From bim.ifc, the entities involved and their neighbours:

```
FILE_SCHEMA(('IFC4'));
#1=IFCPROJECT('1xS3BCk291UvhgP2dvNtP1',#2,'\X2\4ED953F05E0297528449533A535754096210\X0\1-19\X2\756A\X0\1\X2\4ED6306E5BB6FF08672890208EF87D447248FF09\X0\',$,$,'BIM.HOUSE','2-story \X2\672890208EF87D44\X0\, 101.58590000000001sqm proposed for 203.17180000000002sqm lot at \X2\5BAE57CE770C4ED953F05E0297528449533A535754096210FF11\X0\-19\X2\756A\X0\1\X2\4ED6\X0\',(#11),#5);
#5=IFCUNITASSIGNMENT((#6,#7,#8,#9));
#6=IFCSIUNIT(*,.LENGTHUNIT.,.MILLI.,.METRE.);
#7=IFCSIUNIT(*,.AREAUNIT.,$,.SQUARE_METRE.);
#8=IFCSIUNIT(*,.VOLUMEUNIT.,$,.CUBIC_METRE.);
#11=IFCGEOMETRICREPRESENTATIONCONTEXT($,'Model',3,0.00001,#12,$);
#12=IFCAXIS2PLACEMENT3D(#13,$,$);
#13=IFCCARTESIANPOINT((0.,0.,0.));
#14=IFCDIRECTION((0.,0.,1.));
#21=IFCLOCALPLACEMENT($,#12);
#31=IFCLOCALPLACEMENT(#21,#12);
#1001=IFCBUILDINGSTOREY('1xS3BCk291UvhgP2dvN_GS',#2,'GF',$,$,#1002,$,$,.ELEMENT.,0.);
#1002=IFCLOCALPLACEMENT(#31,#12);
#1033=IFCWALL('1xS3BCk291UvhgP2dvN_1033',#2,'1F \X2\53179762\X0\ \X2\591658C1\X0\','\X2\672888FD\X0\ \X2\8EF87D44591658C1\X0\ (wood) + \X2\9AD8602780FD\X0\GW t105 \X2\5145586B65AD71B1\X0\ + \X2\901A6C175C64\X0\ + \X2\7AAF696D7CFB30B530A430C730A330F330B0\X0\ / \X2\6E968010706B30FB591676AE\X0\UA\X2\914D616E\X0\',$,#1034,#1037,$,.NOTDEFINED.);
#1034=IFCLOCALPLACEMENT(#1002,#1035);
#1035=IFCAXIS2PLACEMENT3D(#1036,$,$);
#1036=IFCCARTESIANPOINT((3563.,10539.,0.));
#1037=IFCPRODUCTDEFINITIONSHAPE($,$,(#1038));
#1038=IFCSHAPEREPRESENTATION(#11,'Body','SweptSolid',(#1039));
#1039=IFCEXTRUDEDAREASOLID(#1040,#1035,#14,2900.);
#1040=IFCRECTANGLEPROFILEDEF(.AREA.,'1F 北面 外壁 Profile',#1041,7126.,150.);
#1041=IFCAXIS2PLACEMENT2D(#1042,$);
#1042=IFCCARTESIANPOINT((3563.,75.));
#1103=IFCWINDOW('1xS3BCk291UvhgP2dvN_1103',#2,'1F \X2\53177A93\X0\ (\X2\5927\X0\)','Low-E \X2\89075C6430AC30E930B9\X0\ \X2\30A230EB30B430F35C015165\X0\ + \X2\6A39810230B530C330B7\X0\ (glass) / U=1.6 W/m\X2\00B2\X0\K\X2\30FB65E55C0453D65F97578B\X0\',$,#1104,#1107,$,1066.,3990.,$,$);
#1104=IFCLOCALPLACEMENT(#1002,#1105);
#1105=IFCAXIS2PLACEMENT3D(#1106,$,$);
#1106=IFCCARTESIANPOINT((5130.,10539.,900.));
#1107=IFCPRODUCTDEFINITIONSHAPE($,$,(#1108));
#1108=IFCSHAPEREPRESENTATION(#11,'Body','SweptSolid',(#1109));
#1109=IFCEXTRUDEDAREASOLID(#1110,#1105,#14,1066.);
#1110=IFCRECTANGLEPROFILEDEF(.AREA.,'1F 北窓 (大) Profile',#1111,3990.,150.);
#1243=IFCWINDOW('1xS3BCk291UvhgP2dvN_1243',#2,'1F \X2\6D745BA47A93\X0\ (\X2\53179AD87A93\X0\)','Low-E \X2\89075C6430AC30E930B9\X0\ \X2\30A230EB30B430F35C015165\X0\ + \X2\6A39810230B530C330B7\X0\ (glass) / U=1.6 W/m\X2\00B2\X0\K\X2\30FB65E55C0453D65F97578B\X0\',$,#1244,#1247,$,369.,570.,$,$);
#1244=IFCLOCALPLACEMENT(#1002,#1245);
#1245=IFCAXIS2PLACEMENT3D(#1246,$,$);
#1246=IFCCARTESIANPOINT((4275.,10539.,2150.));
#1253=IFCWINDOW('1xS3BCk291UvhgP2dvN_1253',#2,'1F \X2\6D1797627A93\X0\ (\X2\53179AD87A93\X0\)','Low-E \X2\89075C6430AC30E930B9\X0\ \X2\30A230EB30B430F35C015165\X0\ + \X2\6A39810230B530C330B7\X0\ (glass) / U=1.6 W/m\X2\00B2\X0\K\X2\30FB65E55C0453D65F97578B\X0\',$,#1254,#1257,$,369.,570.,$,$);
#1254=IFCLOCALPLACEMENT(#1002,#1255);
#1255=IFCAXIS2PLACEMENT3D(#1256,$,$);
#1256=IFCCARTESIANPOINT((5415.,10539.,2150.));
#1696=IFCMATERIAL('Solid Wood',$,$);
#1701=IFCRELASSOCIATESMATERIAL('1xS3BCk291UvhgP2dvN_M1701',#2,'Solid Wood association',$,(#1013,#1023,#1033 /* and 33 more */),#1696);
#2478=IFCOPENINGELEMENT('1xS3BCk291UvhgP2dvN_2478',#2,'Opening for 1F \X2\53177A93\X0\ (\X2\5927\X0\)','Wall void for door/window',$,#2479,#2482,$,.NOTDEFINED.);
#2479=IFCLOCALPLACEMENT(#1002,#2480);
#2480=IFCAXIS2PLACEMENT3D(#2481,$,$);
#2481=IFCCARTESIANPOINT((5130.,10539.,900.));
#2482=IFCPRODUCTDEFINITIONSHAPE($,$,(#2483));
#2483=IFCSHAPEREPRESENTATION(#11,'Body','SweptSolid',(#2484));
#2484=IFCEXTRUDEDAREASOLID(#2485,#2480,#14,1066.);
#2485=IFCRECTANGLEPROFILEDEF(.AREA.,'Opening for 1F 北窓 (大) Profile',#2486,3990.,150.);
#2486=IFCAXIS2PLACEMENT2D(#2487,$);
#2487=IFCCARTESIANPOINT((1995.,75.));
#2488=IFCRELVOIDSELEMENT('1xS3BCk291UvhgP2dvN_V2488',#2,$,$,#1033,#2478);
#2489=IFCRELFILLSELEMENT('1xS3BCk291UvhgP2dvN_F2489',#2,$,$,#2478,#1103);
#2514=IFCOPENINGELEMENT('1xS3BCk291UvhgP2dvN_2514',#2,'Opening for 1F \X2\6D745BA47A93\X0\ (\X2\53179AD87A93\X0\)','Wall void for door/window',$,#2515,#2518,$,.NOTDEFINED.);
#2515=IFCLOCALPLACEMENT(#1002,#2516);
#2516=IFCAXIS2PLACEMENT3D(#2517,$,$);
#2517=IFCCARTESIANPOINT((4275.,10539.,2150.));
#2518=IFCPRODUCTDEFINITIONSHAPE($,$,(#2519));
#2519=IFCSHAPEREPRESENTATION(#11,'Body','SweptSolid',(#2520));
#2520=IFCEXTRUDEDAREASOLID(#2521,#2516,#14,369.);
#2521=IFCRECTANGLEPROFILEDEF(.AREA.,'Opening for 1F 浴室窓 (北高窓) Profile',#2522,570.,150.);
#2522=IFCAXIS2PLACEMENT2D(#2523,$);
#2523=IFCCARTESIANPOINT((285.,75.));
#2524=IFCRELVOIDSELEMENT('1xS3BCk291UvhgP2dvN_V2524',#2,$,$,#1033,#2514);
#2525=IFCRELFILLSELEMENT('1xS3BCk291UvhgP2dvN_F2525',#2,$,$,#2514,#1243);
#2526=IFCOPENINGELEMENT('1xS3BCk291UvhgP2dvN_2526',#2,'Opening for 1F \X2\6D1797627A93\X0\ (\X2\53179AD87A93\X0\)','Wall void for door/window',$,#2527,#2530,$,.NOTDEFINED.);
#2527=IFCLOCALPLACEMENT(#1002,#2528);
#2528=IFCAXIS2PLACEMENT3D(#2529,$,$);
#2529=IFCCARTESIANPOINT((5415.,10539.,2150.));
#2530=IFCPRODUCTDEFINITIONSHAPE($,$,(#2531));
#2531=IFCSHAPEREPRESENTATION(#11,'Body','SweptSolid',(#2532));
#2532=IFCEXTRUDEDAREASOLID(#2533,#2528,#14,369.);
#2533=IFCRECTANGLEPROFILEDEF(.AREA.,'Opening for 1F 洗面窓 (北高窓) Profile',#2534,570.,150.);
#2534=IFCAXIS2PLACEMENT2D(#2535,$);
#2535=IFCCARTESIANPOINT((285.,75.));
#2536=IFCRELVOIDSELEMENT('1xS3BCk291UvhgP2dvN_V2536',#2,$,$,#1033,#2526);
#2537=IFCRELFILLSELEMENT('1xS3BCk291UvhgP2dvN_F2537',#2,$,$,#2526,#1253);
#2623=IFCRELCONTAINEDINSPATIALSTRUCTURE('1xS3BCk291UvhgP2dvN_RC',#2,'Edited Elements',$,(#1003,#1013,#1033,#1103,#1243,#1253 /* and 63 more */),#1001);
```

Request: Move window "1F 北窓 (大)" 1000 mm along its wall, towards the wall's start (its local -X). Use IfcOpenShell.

```python
import ifcopenshell
import ifcopenshell.api.geometry
import ifcopenshell.util.placement
import ifcopenshell.util.unit

model = ifcopenshell.open("bim.ifc")
unit_scale = ifcopenshell.util.unit.calculate_unit_scale(model)

window = model.by_guid("1xS3BCk291UvhgP2dvN_1103")
opening = window.FillsVoids[0].RelatingOpeningElement
wall = opening.VoidsElements[0].RelatingBuildingElement

wall_matrix = ifcopenshell.util.placement.get_local_placement(wall.ObjectPlacement)
shift = wall_matrix[:3, 0] * -1 / unit_scale
before = ifcopenshell.util.placement.get_local_placement(window.ObjectPlacement)[:3, 3].copy()

# The window is not placed relative to its opening, so move both.
for product in (opening, window):
    matrix = ifcopenshell.util.placement.get_local_placement(product.ObjectPlacement)
    matrix[:3, 3] += shift
    ifcopenshell.api.geometry.edit_object_placement(model, product=product, matrix=matrix, is_si=False)

after = ifcopenshell.util.placement.get_local_placement(window.ObjectPlacement)[:3, 3]
print("window moved by", (after - before).round(3) + 0.0)

model.write("bim_edited.ifc")
```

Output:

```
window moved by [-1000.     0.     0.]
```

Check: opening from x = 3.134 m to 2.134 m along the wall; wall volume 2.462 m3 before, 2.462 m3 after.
